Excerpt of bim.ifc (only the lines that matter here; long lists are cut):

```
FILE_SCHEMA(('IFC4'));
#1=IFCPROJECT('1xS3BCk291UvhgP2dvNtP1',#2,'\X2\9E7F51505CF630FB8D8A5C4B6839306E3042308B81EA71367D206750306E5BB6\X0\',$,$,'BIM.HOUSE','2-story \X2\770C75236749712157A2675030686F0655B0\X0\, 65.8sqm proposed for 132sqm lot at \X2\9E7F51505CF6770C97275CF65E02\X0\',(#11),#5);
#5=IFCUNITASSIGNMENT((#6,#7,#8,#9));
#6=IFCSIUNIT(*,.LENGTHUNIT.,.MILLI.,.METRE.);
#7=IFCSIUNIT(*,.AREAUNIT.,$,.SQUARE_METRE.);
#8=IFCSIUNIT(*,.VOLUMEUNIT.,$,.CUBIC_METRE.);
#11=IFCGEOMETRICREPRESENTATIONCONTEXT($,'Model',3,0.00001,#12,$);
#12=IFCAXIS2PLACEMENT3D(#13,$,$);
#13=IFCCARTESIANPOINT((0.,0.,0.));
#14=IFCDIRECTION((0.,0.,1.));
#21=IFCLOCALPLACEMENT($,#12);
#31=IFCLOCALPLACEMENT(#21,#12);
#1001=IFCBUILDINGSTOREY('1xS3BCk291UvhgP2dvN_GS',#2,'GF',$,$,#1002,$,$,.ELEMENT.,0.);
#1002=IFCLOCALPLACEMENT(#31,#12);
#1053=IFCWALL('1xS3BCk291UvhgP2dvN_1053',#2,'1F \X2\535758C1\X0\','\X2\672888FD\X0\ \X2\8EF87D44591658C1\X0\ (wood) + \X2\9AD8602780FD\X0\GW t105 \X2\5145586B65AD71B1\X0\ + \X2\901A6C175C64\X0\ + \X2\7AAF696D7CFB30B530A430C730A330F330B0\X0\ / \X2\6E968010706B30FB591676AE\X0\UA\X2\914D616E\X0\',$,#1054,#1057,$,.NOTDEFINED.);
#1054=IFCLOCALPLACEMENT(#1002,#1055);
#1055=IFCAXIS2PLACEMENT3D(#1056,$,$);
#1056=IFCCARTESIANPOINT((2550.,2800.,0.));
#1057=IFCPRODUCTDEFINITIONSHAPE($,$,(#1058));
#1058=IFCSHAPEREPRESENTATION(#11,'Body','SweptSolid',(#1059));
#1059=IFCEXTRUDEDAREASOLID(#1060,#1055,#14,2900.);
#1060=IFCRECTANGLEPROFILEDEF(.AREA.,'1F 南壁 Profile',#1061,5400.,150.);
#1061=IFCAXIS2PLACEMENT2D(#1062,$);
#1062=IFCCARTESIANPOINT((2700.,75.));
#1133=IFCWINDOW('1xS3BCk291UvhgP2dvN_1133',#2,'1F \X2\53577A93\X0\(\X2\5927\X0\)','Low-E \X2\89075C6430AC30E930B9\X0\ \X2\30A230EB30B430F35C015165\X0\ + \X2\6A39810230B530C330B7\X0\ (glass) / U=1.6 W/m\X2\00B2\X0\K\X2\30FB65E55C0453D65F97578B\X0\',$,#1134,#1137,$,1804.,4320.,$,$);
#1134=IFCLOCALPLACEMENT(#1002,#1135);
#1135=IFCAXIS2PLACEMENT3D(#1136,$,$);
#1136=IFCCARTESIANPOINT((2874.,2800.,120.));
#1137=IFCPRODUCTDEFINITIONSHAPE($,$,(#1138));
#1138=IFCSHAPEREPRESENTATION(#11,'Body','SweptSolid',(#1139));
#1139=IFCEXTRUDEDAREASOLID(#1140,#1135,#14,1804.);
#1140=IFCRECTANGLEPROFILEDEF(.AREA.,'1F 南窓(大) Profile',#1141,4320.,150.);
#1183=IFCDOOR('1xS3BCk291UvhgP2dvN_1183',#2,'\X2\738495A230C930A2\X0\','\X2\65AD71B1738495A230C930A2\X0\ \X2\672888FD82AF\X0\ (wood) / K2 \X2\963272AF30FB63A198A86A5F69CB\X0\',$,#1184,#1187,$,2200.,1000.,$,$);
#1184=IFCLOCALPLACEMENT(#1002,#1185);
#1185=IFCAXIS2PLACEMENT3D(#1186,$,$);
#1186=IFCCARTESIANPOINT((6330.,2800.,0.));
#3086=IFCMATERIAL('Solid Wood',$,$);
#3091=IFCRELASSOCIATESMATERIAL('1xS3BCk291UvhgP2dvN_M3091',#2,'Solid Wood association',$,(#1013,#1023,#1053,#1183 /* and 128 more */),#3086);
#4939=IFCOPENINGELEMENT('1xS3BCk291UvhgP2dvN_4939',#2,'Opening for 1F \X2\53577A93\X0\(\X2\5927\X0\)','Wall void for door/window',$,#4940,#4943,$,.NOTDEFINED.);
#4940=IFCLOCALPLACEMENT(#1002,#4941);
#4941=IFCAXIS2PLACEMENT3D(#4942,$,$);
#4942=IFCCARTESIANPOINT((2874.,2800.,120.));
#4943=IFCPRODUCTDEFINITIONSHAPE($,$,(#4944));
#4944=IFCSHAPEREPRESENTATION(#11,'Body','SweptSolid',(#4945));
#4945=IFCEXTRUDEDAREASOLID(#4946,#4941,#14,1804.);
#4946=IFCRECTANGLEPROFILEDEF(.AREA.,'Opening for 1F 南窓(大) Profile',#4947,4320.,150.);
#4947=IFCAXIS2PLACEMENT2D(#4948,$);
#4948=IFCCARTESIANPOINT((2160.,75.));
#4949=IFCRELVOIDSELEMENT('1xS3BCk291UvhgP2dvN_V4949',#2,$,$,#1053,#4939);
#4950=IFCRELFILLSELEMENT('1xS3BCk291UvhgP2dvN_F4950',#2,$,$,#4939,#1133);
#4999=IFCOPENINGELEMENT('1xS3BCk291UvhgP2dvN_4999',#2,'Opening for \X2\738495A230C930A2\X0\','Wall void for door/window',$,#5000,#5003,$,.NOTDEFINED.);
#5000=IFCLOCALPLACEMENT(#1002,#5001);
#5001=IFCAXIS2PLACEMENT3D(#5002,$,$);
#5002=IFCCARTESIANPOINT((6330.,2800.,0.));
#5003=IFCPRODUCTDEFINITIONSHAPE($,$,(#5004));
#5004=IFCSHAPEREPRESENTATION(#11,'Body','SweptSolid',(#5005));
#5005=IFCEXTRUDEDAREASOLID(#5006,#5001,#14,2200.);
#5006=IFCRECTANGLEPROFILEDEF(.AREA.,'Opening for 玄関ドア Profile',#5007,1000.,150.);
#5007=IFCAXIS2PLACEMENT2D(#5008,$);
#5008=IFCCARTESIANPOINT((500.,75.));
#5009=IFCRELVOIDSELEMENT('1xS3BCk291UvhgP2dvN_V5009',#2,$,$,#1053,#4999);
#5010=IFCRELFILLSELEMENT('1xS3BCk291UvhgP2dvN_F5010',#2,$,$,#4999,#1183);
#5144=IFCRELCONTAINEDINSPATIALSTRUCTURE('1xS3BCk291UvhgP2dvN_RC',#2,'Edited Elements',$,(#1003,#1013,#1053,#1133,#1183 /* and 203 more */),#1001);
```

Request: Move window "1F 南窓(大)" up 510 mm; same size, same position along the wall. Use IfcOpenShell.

```python
import numpy as np
import ifcopenshell
import ifcopenshell.api.geometry
import ifcopenshell.util.placement
import ifcopenshell.util.unit

model = ifcopenshell.open("bim.ifc")
unit_scale = ifcopenshell.util.unit.calculate_unit_scale(model)

window = model.by_id(1133)
opening = window.FillsVoids[0].RelatingOpeningElement
dz = 510.0

shift = np.array([0.0, 0.0, dz])
# The window is not placed relative to its opening, so move both.
for product in (opening, window):
    matrix = ifcopenshell.util.placement.get_local_placement(product.ObjectPlacement)
    matrix[:3, 3] += shift
    ifcopenshell.api.geometry.edit_object_placement(model, product=product, matrix=matrix, is_si=False)

print(f"moved by {dz * unit_scale:+.3f} m")

model.write("bim_updated.ifc")
```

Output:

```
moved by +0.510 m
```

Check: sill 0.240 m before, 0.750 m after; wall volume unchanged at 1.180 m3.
